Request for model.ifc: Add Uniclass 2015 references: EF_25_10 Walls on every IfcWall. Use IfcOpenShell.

First a look at what the model holds.

```python
import ifcopenshell

model = ifcopenshell.open("model.ifc")
print(model.schema)
print("classifications:", [c.Name for c in model.by_type("IfcClassification")])
for ifc_class in ("IfcDoor", "IfcRoof", "IfcStair", "IfcWall", "IfcWindow"):
    print(ifc_class, len(model.by_type(ifc_class)))
```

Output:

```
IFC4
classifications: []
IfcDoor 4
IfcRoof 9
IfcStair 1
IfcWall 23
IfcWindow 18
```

```python
import ifcopenshell
import ifcopenshell.api.classification

model = ifcopenshell.open("model.ifc")

system = ifcopenshell.api.classification.add_classification(model, classification="Uniclass 2015")

codes = {
    "IfcWall": ("EF_25_10", "Walls"),
}
for ifc_class, (code, name) in codes.items():
    products = model.by_type(ifc_class)
    ifcopenshell.api.classification.add_reference(
        model, products=products, classification=system, identification=code, name=name
    )
    print(code, len(products))

model.write("model_v2.ifc")
```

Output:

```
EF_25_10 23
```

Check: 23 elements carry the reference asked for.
